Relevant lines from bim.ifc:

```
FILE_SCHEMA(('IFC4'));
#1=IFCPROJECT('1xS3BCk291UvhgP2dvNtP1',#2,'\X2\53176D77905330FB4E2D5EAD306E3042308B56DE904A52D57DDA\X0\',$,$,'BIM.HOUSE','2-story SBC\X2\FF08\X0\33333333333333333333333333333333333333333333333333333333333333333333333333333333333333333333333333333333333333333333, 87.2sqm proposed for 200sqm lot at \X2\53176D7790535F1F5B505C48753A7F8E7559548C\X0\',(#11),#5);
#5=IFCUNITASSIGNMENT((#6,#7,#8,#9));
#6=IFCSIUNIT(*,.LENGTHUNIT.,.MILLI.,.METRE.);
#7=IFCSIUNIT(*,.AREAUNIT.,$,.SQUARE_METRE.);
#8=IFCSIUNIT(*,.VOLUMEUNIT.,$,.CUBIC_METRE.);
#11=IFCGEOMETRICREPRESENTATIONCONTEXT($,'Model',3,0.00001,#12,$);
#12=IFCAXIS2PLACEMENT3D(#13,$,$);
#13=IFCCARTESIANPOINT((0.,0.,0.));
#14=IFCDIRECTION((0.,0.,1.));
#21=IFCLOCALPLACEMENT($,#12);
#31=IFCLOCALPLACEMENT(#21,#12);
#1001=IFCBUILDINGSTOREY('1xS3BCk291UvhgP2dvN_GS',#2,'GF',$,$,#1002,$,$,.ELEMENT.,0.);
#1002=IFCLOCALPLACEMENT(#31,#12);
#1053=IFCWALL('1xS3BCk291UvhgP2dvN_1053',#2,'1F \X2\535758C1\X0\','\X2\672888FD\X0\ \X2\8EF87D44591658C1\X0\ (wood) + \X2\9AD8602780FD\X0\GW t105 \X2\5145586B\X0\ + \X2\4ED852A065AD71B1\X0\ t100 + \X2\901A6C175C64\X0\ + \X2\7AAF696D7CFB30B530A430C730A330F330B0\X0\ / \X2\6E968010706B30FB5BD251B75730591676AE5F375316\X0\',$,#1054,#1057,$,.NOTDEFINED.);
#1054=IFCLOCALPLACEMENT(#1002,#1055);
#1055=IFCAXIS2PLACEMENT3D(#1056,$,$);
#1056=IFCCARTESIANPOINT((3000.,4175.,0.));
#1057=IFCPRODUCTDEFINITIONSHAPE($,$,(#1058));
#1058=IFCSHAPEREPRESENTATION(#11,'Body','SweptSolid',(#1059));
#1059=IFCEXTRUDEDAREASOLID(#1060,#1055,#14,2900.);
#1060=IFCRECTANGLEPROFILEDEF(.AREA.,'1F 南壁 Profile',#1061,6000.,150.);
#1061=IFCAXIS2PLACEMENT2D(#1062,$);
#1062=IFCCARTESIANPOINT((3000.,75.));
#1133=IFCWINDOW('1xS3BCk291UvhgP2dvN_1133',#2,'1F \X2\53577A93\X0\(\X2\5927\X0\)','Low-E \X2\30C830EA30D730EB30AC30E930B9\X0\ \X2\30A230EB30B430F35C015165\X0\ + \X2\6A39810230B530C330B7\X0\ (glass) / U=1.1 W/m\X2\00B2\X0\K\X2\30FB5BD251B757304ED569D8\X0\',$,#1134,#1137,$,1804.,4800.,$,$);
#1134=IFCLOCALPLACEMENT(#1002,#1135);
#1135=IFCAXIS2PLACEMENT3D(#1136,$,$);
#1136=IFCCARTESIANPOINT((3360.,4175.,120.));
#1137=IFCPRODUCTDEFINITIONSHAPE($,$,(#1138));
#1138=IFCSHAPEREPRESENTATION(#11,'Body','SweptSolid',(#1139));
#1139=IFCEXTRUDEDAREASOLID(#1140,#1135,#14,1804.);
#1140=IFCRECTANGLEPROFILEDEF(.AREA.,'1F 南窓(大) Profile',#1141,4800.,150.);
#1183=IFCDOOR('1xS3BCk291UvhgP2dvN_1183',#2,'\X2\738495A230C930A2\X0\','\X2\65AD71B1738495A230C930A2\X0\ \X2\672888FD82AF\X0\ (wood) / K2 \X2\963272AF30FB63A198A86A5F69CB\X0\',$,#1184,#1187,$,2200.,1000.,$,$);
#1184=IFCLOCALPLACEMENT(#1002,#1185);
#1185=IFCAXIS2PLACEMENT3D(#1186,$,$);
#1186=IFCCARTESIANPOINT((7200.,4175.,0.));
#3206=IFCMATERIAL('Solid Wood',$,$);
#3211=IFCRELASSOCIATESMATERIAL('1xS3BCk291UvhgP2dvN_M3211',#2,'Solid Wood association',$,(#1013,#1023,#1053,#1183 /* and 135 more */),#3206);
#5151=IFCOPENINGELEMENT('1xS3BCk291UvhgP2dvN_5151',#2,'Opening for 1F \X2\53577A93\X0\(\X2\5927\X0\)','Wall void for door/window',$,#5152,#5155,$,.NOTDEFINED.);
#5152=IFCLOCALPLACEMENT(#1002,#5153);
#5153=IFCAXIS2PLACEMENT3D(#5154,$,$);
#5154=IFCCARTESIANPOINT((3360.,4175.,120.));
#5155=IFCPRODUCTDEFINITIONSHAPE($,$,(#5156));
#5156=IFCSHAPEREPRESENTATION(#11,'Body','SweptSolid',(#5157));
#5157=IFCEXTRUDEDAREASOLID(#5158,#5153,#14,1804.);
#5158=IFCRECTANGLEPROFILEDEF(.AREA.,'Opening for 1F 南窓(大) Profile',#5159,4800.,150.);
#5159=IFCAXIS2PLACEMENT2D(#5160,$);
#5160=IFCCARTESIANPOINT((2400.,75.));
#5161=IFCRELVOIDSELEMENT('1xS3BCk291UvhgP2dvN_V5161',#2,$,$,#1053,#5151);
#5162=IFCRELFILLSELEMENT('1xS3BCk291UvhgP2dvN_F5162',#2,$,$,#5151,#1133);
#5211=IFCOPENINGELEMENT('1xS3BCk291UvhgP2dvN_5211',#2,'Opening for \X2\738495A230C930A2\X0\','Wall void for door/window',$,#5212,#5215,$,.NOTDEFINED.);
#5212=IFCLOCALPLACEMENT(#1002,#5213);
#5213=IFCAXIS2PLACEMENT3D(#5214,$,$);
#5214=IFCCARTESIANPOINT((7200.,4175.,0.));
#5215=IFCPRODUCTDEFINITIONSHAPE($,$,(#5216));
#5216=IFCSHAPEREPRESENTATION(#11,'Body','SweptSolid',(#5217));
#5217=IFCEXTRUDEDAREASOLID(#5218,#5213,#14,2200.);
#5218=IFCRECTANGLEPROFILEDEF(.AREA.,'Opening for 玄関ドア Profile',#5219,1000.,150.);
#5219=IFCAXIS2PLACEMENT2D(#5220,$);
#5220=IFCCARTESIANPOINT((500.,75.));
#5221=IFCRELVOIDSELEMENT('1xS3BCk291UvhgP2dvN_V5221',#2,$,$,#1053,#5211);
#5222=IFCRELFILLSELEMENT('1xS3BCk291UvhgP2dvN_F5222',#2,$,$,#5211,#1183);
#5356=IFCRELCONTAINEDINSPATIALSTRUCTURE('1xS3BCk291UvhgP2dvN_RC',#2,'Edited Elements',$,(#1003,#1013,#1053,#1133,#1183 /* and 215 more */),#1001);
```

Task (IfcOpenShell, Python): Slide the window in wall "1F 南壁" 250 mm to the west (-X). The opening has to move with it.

```python
import ifcopenshell
import ifcopenshell.api.geometry
import ifcopenshell.util.placement
import ifcopenshell.util.unit

model = ifcopenshell.open("bim.ifc")
unit_scale = ifcopenshell.util.unit.calculate_unit_scale(model)

window = model.by_id(1133)
opening = window.FillsVoids[0].RelatingOpeningElement
wall = opening.VoidsElements[0].RelatingBuildingElement

wall_matrix = ifcopenshell.util.placement.get_local_placement(wall.ObjectPlacement)
shift = wall_matrix[:3, 0] * -0.25 / unit_scale
before = ifcopenshell.util.placement.get_local_placement(window.ObjectPlacement)[:3, 3].copy()

# The window is not placed relative to its opening, so move both.
for product in (opening, window):
    matrix = ifcopenshell.util.placement.get_local_placement(product.ObjectPlacement)
    matrix[:3, 3] += shift
    ifcopenshell.api.geometry.edit_object_placement(model, product=product, matrix=matrix, is_si=False)

after = ifcopenshell.util.placement.get_local_placement(window.ObjectPlacement)[:3, 3]
print("window moved by", (after - before).round(3) + 0.0)

model.write("bim_rev.ifc")
```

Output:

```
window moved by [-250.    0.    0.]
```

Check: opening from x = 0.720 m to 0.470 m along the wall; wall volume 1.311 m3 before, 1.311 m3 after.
